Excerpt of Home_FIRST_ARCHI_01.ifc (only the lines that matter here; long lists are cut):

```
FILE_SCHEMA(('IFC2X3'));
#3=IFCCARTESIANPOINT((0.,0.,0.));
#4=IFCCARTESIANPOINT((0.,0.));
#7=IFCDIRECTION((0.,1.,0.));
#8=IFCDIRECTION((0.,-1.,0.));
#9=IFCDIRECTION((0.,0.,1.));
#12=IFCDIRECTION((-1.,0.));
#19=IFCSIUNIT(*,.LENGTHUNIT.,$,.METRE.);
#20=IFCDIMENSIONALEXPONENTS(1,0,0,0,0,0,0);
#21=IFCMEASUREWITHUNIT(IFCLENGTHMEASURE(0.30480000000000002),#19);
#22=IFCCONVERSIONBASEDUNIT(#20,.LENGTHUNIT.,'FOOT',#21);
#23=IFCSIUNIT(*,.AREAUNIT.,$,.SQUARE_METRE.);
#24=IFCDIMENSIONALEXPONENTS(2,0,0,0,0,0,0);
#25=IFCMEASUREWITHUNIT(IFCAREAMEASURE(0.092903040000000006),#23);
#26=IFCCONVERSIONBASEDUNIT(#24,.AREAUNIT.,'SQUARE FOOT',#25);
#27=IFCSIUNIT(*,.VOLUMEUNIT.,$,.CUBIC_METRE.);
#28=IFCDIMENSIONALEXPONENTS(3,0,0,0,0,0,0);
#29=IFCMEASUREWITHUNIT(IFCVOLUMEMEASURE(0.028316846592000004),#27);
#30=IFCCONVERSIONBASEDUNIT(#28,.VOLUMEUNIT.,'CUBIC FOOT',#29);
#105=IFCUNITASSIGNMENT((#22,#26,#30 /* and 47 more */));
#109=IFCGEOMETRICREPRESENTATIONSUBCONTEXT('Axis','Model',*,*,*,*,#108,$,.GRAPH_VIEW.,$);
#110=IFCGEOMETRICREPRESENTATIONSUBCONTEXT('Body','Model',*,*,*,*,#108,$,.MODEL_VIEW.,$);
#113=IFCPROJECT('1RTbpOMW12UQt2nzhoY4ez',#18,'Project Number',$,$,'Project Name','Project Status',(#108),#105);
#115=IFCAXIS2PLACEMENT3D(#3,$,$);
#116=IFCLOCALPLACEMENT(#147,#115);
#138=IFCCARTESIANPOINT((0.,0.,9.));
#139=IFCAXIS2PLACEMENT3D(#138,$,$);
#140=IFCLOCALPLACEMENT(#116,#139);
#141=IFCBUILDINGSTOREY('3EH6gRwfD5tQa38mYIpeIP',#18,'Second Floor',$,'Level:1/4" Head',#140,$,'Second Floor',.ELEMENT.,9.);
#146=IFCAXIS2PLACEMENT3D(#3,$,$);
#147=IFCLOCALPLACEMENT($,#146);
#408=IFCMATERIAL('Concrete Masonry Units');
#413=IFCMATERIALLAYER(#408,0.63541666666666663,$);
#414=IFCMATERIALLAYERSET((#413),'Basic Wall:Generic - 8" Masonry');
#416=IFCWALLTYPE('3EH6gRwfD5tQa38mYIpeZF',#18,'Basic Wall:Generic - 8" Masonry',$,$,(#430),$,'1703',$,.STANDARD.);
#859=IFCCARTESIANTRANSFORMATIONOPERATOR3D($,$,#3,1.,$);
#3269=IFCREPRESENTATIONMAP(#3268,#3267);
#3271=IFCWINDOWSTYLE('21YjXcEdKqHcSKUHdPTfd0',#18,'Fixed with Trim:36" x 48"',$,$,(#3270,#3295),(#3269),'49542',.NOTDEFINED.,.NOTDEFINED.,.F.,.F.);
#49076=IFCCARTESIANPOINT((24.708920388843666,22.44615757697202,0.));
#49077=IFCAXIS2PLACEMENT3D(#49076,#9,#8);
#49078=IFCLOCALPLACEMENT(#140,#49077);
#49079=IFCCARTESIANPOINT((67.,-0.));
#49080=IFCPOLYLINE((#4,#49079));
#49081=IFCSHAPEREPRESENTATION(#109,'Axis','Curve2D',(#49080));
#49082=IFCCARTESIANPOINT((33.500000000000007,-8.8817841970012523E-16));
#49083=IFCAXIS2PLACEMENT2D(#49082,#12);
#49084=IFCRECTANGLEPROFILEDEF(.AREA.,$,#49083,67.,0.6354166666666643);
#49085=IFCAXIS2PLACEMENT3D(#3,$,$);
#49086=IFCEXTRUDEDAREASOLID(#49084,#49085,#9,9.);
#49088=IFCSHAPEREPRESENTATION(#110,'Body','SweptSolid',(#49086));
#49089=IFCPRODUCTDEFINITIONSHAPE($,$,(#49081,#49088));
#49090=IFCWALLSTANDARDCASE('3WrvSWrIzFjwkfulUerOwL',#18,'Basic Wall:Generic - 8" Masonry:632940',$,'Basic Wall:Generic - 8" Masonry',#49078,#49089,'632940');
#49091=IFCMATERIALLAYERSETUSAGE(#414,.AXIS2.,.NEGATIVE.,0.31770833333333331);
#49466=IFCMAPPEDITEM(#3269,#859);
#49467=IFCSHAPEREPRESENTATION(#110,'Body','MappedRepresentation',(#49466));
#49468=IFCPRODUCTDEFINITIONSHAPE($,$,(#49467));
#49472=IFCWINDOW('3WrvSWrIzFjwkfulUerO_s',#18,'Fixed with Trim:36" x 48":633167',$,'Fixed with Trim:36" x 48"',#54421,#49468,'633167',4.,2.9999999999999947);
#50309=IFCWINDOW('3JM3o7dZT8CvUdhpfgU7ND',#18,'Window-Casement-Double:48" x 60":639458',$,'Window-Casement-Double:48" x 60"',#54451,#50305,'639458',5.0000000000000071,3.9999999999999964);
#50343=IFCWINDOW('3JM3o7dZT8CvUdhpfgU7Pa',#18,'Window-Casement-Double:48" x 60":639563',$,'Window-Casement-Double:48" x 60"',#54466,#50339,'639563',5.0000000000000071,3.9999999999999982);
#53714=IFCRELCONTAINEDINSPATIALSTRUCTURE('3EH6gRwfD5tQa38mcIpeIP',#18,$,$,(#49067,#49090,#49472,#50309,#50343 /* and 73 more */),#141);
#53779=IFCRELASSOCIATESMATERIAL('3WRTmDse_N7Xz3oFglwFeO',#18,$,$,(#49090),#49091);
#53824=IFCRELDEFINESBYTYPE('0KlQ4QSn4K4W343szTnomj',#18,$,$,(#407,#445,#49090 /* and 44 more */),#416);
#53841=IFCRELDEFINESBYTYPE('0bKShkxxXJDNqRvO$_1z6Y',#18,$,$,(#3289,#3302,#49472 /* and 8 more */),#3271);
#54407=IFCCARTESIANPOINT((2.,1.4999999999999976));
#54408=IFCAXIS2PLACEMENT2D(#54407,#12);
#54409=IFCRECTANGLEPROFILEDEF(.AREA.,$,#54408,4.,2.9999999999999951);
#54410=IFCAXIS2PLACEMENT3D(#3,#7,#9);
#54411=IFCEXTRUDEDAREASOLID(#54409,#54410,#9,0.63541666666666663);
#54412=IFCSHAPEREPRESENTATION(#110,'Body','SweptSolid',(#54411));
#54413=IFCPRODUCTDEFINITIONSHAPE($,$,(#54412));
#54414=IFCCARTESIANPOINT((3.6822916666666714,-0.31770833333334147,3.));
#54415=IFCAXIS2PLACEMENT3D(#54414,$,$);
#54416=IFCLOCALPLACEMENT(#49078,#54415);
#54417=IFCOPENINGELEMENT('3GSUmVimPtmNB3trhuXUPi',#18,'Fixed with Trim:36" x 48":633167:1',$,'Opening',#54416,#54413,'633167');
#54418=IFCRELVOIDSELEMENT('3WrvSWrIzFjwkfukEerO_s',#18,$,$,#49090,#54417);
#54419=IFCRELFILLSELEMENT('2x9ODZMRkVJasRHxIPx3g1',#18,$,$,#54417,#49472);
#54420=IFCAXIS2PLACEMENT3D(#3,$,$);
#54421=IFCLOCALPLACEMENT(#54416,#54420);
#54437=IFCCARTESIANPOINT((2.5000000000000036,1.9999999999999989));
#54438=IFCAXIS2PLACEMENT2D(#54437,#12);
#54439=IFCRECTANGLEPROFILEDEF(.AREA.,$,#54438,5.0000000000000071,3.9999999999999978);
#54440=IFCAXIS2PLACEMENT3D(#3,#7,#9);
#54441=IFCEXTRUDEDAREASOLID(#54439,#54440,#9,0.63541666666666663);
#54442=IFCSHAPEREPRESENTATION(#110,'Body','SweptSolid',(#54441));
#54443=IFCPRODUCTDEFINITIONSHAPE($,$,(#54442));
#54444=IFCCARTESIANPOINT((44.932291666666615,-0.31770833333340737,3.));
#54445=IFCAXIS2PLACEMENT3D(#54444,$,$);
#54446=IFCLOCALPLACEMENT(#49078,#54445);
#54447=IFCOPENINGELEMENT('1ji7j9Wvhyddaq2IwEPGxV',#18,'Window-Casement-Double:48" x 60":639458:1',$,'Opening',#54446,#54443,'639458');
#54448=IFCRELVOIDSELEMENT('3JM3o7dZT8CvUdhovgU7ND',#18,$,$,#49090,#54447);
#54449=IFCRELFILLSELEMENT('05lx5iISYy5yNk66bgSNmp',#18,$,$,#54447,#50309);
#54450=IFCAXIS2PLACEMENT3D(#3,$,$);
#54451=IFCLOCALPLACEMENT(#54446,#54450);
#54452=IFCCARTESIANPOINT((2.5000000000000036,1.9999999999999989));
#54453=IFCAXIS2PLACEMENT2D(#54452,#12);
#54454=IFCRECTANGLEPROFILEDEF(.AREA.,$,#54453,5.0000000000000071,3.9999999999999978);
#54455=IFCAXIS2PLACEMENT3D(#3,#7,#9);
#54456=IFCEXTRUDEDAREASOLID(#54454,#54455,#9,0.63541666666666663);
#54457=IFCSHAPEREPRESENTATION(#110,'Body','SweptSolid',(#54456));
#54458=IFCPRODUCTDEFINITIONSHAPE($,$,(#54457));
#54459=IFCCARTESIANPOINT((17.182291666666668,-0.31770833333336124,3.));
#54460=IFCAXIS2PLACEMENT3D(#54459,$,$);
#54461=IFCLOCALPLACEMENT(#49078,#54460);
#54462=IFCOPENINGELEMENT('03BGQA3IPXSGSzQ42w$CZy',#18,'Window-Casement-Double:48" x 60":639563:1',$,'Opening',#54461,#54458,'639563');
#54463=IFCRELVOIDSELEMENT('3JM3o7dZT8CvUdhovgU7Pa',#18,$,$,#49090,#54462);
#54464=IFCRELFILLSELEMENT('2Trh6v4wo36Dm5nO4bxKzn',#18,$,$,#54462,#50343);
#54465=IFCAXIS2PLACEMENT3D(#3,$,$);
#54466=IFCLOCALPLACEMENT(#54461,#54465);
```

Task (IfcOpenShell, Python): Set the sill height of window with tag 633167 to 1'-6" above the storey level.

```python
import numpy as np
import ifcopenshell
import ifcopenshell.api.geometry
import ifcopenshell.geom
import ifcopenshell.util.element
import ifcopenshell.util.placement
import ifcopenshell.util.shape
import ifcopenshell.util.unit

model = ifcopenshell.open("Home_FIRST_ARCHI_01.ifc")
unit_scale = ifcopenshell.util.unit.calculate_unit_scale(model)

window = model.by_guid("3WrvSWrIzFjwkfulUerO_s")
opening = window.FillsVoids[0].RelatingOpeningElement
storey = ifcopenshell.util.element.get_container(window, ifc_class="IfcBuildingStorey")
level = ifcopenshell.util.placement.get_local_placement(storey.ObjectPlacement)[2, 3]

# The opening's origin need not be at the sill, so measure its lowest point.
shape = ifcopenshell.geom.create_shape(ifcopenshell.geom.settings(), opening)
bottom = ifcopenshell.util.shape.get_shape_bottom_elevation(shape, shape.geometry) / unit_scale
dz = level + 18 * 0.0254 / unit_scale - bottom

shift = np.array([0.0, 0.0, dz])
# The window is placed relative to its opening, so it follows when the opening moves.
matrix = ifcopenshell.util.placement.get_local_placement(opening.ObjectPlacement)
matrix[:3, 3] += shift
ifcopenshell.api.geometry.edit_object_placement(
    model, product=opening, matrix=matrix, is_si=False, should_transform_children=True
)

print(f"moved by {dz * unit_scale:+.3f} m")

model.write("Home_FIRST_ARCHI_01_v2.ifc")
```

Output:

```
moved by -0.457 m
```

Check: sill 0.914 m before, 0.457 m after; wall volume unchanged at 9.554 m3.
